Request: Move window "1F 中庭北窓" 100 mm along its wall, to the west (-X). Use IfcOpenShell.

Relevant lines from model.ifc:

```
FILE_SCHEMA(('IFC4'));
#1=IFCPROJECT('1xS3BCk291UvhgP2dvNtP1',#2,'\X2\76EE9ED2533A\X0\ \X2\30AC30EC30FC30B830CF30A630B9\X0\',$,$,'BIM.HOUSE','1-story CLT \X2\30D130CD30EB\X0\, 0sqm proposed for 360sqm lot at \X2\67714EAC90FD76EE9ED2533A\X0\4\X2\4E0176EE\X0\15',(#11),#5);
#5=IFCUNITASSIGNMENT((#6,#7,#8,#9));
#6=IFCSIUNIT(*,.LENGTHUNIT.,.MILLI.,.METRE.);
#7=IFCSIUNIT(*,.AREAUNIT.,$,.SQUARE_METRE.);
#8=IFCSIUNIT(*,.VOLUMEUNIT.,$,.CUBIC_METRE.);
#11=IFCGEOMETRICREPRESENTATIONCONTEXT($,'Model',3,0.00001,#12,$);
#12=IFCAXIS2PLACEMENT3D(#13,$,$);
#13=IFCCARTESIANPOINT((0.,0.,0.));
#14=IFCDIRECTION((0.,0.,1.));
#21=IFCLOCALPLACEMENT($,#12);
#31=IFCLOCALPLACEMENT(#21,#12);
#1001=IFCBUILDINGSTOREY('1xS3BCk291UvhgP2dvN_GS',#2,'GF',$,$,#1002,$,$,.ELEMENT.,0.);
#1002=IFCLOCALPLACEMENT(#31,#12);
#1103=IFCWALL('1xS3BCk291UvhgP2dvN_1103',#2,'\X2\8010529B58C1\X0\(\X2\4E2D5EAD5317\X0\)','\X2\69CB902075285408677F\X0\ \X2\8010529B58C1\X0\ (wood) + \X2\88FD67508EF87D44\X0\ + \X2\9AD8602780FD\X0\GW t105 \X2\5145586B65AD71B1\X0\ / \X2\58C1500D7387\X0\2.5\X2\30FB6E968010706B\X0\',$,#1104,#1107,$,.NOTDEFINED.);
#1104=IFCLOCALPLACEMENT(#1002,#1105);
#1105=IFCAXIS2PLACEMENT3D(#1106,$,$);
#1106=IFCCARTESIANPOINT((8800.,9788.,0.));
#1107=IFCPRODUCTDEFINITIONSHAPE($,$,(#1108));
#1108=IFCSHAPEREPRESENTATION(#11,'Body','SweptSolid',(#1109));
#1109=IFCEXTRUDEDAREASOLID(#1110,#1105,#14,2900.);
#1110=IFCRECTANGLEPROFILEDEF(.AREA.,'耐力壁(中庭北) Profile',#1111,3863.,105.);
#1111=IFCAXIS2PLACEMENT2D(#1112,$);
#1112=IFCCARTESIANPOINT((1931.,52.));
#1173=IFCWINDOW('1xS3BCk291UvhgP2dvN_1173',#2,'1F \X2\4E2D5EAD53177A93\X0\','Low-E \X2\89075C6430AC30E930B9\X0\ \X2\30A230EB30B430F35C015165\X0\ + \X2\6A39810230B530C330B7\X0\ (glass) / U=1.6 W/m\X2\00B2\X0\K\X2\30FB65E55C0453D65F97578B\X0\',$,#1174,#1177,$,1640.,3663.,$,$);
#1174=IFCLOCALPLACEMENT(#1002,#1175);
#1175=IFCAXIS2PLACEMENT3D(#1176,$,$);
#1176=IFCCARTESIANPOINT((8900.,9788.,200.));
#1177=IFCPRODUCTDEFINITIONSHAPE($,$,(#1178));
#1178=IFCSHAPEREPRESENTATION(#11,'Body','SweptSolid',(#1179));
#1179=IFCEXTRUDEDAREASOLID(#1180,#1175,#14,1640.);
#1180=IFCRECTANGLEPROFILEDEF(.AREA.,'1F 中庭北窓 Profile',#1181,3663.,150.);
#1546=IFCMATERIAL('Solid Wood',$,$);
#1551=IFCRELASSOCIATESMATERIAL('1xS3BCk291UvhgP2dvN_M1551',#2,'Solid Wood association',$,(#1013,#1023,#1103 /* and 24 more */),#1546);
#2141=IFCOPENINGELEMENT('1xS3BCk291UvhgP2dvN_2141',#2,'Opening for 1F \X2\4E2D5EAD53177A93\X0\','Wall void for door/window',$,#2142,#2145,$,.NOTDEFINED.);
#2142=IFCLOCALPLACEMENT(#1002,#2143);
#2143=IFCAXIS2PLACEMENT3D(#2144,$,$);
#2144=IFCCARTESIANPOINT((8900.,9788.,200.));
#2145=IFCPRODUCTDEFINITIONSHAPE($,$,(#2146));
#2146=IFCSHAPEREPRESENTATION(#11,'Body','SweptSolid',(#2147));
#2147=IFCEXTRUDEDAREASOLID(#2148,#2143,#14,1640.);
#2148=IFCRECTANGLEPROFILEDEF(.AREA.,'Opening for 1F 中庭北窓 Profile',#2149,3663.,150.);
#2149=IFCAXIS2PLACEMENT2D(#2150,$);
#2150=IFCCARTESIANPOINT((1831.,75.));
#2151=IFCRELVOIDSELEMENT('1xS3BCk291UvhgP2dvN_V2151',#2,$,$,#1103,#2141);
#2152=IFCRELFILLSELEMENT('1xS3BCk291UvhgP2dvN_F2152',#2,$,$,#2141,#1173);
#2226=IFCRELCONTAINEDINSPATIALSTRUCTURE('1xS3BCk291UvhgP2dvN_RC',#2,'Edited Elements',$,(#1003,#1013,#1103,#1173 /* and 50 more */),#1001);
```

```python
import ifcopenshell
import ifcopenshell.api.geometry
import ifcopenshell.util.placement
import ifcopenshell.util.unit

model = ifcopenshell.open("model.ifc")
unit_scale = ifcopenshell.util.unit.calculate_unit_scale(model)

window = model.by_id(1173)
opening = window.FillsVoids[0].RelatingOpeningElement
wall = opening.VoidsElements[0].RelatingBuildingElement

wall_matrix = ifcopenshell.util.placement.get_local_placement(wall.ObjectPlacement)
shift = wall_matrix[:3, 0] * -0.1 / unit_scale
before = ifcopenshell.util.placement.get_local_placement(window.ObjectPlacement)[:3, 3].copy()

# The window is not placed relative to its opening, so move both.
for product in (opening, window):
    matrix = ifcopenshell.util.placement.get_local_placement(product.ObjectPlacement)
    matrix[:3, 3] += shift
    ifcopenshell.api.geometry.edit_object_placement(model, product=product, matrix=matrix, is_si=False)

after = ifcopenshell.util.placement.get_local_placement(window.ObjectPlacement)[:3, 3]
print("window moved by", (after - before).round(3) + 0.0)

model.write("model_rev.ifc")
```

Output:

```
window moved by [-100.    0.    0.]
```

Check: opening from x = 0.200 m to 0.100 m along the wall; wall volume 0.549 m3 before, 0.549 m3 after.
